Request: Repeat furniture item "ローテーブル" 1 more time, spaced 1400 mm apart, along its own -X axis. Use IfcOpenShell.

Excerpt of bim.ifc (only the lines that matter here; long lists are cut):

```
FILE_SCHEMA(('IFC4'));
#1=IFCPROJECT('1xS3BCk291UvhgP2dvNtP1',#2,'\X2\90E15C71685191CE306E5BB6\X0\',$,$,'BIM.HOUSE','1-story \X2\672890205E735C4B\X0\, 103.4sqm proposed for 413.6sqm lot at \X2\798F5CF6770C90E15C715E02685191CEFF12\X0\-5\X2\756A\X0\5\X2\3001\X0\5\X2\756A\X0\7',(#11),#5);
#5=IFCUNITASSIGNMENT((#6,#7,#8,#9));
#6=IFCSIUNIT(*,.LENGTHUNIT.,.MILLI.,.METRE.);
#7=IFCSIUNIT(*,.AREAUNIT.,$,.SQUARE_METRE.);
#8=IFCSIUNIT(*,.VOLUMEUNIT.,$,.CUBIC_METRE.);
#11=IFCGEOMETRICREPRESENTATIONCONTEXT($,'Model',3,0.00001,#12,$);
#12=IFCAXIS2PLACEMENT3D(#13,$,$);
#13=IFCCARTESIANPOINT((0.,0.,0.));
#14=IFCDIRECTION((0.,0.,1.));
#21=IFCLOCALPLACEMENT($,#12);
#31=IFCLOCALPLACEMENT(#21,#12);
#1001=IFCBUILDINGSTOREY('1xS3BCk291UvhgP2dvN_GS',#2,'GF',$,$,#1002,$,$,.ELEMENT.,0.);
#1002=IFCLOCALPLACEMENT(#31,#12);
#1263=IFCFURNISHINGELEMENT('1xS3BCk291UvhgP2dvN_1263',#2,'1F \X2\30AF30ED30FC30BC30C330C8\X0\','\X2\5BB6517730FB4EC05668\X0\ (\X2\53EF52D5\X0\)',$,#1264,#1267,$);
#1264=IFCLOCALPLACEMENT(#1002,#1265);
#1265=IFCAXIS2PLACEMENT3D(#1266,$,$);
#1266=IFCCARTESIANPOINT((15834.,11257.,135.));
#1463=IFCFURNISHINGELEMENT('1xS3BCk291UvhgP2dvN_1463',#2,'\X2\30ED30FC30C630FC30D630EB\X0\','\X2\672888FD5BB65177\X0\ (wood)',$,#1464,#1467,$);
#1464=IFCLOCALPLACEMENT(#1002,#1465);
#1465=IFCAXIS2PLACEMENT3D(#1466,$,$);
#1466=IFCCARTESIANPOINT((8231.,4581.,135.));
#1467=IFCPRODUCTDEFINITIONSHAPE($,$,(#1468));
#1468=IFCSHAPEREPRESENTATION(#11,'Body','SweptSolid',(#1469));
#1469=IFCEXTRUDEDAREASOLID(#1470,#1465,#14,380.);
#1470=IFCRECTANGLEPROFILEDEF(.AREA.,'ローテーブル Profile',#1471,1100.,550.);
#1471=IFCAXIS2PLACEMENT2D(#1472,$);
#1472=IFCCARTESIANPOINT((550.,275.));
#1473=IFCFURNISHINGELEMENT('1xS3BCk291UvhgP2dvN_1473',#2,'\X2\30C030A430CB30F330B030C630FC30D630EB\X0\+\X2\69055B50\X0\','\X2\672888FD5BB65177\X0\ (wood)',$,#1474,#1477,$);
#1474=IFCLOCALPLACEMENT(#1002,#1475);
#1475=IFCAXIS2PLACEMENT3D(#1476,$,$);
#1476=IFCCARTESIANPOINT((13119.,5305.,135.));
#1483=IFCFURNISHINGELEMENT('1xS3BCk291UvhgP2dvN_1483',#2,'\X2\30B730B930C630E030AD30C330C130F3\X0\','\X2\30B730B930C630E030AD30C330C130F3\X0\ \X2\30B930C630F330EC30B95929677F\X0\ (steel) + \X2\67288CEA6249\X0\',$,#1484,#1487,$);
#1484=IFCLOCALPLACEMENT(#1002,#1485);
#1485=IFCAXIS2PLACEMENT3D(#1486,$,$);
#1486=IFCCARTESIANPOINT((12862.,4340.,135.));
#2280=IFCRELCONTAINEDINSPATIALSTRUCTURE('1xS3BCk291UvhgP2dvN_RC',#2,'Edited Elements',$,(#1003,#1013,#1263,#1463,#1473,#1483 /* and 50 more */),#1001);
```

```python
import ifcopenshell
import ifcopenshell.api.geometry
import ifcopenshell.api.root
import ifcopenshell.util.element
import ifcopenshell.util.placement
import ifcopenshell.util.unit

model = ifcopenshell.open("bim.ifc")
unit_scale = ifcopenshell.util.unit.calculate_unit_scale(model)


def reuse_history(source, copy):
    """copy_class also copies each property set's owner history, people and application; keep the originals."""
    for rel in copy.IsDefinedBy:
        if rel.is_a("IfcRelDefinesByProperties") and (history := rel.RelatingPropertyDefinition.OwnerHistory):
            rel.RelatingPropertyDefinition.OwnerHistory = source.OwnerHistory
            ifcopenshell.util.element.remove_deep2(model, history)


source = model.by_guid("1xS3BCk291UvhgP2dvN_1463")
base = ifcopenshell.util.placement.get_local_placement(source.ObjectPlacement)
step = -base[:3, 0] * 1.4 / unit_scale

for i in range(1, 2):
    copy = ifcopenshell.api.root.copy_class(model, product=source)
    copy.Representation = ifcopenshell.util.element.copy_deep(
        model, source.Representation, exclude=["IfcGeometricRepresentationContext", "IfcRepresentationMap"]
    )
    reuse_history(source, copy)
    matrix = base.copy()
    matrix[:3, 3] += i * step
    print("added at", matrix[:3, 3].round(3) + 0.0)
    ifcopenshell.api.geometry.edit_object_placement(model, product=copy, matrix=matrix, is_si=False)

model.write("bim_edited.ifc")
```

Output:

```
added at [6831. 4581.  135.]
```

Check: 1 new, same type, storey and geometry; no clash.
